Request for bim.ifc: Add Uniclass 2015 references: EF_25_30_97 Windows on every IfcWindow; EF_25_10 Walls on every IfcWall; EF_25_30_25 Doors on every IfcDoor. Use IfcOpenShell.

First a look at what the model holds.

```python
import ifcopenshell

model = ifcopenshell.open("bim.ifc")
print(model.schema)
print("classifications:", [c.Name for c in model.by_type("IfcClassification")])
for ifc_class in ("IfcDoor", "IfcRoof", "IfcStair", "IfcWall", "IfcWindow"):
    print(ifc_class, len(model.by_type(ifc_class)))
```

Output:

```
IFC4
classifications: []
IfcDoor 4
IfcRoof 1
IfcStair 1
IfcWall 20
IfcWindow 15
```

```python
import ifcopenshell
import ifcopenshell.api.classification

model = ifcopenshell.open("bim.ifc")

system = ifcopenshell.api.classification.add_classification(model, classification="Uniclass 2015")

codes = {
    "IfcWindow": ("EF_25_30_97", "Windows"),
    "IfcWall": ("EF_25_10", "Walls"),
    "IfcDoor": ("EF_25_30_25", "Doors"),
}
for ifc_class, (code, name) in codes.items():
    products = model.by_type(ifc_class)
    ifcopenshell.api.classification.add_reference(
        model, products=products, classification=system, identification=code, name=name
    )
    print(code, len(products))

model.write("bim_edited.ifc")
```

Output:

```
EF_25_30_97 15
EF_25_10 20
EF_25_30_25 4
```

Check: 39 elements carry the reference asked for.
